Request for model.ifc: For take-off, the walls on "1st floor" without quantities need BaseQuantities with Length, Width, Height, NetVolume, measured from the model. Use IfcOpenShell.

First a look at what the model holds.

```python
import ifcopenshell
import ifcopenshell.util.element
import ifcopenshell.util.unit

model = ifcopenshell.open("model.ifc")
print(model.schema)
for unit_type in ("LENGTHUNIT", "AREAUNIT", "VOLUMEUNIT"):
    print(unit_type, ifcopenshell.util.unit.calculate_unit_scale(model, unit_type))
storey = next(s for s in model.by_type("IfcBuildingStorey") if s.Name == "1st floor")
walls = [e for e in ifcopenshell.util.element.get_decomposition(storey) if e.is_a("IfcWall")]
for e in sorted(walls, key=lambda e: e.id()):
    print(e.id(), e.is_a(), e.Name, list(ifcopenshell.util.element.get_psets(e, qtos_only=True)), sep=" | ")
```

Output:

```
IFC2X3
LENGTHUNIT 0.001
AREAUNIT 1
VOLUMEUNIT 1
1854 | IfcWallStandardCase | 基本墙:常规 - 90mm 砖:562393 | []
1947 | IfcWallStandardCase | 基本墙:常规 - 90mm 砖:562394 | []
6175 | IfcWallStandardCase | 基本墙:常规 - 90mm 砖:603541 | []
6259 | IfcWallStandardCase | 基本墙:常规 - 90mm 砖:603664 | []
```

```python
import ifcopenshell
import ifcopenshell.api.pset
import ifcopenshell.geom
import ifcopenshell.util.element
import ifcopenshell.util.shape
import ifcopenshell.util.unit

model = ifcopenshell.open("model.ifc")
unit_scale = ifcopenshell.util.unit.calculate_unit_scale(model)
volume_scale = ifcopenshell.util.unit.calculate_unit_scale(model, "VOLUMEUNIT")
settings = ifcopenshell.geom.settings()

storey = next(s for s in model.by_type("IfcBuildingStorey") if s.Name == "1st floor")
walls = [e for e in ifcopenshell.util.element.get_decomposition(storey) if e.is_a("IfcWall")]

for e in sorted(walls, key=lambda e: e.id()):
    if ifcopenshell.util.element.get_psets(e, qtos_only=True, should_inherit=False):
        continue
    # Geometry comes back in metres, in the element's own axes.
    shape = ifcopenshell.geom.create_shape(settings, e)
    values = {
        "Length": ifcopenshell.util.shape.get_x(shape.geometry) / unit_scale,
        "Width": ifcopenshell.util.shape.get_y(shape.geometry) / unit_scale,
        "Height": ifcopenshell.util.shape.get_z(shape.geometry) / unit_scale,
        "NetVolume": ifcopenshell.util.shape.get_volume(shape.geometry) / volume_scale,
    }
    qto = ifcopenshell.api.pset.add_qto(model, product=e, name="BaseQuantities")
    ifcopenshell.api.pset.edit_qto(model, qto=qto, properties=values)
    print(e.id(), {k: round(v, 3) for k, v in values.items()})

model.write("model-out.ifc")
```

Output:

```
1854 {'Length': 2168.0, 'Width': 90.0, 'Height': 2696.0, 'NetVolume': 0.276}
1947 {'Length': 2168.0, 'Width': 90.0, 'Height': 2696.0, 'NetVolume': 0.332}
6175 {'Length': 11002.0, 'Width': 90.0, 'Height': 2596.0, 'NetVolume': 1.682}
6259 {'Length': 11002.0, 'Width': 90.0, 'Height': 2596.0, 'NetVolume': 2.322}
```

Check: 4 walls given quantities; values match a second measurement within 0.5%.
